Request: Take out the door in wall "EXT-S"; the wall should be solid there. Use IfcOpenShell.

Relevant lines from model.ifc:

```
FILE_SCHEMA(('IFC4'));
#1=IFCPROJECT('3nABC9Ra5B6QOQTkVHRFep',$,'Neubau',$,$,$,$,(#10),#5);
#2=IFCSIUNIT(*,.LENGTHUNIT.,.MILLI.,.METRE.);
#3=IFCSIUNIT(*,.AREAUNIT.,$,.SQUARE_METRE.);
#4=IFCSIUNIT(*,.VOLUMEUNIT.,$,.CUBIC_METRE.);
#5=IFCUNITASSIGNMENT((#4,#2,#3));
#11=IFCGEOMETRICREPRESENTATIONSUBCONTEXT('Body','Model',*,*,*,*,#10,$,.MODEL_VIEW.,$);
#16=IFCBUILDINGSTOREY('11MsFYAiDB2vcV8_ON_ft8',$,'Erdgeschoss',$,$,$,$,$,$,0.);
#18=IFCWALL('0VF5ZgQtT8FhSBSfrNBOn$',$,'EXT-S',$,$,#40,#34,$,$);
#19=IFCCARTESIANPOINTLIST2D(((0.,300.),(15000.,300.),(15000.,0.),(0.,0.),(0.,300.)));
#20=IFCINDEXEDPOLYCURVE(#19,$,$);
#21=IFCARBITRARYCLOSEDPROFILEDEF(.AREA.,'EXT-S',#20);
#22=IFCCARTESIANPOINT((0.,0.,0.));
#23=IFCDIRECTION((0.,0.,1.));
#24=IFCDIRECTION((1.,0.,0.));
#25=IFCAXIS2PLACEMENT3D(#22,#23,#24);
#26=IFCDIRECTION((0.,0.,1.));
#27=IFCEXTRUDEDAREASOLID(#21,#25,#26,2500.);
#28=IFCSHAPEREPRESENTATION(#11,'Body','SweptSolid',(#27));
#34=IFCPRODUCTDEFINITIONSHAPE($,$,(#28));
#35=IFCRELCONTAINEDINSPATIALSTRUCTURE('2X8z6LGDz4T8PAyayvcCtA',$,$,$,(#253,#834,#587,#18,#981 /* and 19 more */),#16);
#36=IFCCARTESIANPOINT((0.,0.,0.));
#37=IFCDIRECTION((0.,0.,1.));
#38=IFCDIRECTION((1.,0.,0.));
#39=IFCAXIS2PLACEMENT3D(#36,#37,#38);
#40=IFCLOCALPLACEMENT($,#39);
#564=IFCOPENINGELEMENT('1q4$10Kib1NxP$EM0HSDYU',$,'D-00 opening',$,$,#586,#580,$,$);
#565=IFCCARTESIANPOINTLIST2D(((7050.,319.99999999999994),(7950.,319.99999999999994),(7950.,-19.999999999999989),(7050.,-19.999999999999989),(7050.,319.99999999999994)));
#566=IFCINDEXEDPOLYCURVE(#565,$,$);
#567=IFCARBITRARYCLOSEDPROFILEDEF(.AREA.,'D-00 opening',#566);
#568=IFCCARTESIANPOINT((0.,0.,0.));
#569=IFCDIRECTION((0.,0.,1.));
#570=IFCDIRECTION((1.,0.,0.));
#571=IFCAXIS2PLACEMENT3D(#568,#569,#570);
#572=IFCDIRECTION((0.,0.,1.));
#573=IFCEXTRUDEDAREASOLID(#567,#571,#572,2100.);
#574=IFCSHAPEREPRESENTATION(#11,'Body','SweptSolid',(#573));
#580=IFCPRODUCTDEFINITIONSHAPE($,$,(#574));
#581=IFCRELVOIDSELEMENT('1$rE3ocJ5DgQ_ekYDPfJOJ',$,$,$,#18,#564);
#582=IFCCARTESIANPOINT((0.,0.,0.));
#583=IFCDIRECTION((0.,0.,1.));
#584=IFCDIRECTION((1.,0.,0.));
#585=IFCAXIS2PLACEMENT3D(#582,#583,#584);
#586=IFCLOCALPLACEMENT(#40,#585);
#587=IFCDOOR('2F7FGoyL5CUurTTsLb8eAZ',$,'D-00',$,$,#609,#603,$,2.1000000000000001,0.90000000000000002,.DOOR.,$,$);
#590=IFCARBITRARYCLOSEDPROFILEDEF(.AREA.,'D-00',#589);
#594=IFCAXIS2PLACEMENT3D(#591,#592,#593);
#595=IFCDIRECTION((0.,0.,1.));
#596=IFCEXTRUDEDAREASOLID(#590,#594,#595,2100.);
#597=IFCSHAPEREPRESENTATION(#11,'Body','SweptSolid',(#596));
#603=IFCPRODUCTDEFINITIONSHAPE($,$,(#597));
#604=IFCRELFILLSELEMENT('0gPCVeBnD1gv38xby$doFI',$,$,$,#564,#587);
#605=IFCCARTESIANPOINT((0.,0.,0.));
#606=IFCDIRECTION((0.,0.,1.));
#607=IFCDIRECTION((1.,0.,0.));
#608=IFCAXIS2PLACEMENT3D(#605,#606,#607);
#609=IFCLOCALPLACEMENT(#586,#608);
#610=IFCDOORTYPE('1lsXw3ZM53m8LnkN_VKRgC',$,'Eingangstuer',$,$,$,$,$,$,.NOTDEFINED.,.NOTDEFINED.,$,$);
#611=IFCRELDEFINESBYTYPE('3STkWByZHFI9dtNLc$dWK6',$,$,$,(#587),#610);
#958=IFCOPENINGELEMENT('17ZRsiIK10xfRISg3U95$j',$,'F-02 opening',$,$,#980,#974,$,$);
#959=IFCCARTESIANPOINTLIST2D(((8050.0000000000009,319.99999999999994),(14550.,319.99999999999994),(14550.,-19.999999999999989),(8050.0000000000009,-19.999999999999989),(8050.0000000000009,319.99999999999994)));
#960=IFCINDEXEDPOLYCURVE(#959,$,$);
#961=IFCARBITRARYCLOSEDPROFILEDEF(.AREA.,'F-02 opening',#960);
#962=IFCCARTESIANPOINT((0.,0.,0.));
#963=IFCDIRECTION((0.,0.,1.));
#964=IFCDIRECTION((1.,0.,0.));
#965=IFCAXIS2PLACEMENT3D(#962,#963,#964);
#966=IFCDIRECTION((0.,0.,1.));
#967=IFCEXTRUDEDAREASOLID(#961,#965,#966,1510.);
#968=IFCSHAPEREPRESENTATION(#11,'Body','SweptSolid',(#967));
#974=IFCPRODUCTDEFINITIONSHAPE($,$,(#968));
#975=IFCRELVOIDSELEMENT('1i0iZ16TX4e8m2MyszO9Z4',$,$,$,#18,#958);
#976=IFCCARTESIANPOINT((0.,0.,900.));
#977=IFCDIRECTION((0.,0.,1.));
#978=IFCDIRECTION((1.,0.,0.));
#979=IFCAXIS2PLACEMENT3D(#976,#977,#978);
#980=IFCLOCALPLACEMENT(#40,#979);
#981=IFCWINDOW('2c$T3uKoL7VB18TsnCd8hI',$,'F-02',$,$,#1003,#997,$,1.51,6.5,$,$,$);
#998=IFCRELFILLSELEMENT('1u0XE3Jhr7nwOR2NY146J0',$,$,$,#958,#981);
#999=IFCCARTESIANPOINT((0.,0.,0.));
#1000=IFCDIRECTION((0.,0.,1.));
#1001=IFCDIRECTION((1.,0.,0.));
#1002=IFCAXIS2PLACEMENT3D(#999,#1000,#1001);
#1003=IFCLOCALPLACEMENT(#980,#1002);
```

```python
import ifcopenshell
import ifcopenshell.api.feature
import ifcopenshell.api.root
import ifcopenshell.geom
import ifcopenshell.util.shape

model = ifcopenshell.open("model.ifc")
settings = ifcopenshell.geom.settings()


def volume(element):
    """Net volume in cubic metres, openings subtracted."""
    shape = ifcopenshell.geom.create_shape(settings, element)
    return ifcopenshell.util.shape.get_volume(shape.geometry)


door = model.by_id(587)
opening = door.FillsVoids[0].RelatingOpeningElement
wall = opening.VoidsElements[0].RelatingBuildingElement
before = volume(wall)

ifcopenshell.api.root.remove_product(model, product=door)
ifcopenshell.api.feature.remove_feature(model, feature=opening)

after = volume(wall)

print(f"wall volume {before:.3f} -> {after:.3f} m3")

model.write("model-out.ifc")
```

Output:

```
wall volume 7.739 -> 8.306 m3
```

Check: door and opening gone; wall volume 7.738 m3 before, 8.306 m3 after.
